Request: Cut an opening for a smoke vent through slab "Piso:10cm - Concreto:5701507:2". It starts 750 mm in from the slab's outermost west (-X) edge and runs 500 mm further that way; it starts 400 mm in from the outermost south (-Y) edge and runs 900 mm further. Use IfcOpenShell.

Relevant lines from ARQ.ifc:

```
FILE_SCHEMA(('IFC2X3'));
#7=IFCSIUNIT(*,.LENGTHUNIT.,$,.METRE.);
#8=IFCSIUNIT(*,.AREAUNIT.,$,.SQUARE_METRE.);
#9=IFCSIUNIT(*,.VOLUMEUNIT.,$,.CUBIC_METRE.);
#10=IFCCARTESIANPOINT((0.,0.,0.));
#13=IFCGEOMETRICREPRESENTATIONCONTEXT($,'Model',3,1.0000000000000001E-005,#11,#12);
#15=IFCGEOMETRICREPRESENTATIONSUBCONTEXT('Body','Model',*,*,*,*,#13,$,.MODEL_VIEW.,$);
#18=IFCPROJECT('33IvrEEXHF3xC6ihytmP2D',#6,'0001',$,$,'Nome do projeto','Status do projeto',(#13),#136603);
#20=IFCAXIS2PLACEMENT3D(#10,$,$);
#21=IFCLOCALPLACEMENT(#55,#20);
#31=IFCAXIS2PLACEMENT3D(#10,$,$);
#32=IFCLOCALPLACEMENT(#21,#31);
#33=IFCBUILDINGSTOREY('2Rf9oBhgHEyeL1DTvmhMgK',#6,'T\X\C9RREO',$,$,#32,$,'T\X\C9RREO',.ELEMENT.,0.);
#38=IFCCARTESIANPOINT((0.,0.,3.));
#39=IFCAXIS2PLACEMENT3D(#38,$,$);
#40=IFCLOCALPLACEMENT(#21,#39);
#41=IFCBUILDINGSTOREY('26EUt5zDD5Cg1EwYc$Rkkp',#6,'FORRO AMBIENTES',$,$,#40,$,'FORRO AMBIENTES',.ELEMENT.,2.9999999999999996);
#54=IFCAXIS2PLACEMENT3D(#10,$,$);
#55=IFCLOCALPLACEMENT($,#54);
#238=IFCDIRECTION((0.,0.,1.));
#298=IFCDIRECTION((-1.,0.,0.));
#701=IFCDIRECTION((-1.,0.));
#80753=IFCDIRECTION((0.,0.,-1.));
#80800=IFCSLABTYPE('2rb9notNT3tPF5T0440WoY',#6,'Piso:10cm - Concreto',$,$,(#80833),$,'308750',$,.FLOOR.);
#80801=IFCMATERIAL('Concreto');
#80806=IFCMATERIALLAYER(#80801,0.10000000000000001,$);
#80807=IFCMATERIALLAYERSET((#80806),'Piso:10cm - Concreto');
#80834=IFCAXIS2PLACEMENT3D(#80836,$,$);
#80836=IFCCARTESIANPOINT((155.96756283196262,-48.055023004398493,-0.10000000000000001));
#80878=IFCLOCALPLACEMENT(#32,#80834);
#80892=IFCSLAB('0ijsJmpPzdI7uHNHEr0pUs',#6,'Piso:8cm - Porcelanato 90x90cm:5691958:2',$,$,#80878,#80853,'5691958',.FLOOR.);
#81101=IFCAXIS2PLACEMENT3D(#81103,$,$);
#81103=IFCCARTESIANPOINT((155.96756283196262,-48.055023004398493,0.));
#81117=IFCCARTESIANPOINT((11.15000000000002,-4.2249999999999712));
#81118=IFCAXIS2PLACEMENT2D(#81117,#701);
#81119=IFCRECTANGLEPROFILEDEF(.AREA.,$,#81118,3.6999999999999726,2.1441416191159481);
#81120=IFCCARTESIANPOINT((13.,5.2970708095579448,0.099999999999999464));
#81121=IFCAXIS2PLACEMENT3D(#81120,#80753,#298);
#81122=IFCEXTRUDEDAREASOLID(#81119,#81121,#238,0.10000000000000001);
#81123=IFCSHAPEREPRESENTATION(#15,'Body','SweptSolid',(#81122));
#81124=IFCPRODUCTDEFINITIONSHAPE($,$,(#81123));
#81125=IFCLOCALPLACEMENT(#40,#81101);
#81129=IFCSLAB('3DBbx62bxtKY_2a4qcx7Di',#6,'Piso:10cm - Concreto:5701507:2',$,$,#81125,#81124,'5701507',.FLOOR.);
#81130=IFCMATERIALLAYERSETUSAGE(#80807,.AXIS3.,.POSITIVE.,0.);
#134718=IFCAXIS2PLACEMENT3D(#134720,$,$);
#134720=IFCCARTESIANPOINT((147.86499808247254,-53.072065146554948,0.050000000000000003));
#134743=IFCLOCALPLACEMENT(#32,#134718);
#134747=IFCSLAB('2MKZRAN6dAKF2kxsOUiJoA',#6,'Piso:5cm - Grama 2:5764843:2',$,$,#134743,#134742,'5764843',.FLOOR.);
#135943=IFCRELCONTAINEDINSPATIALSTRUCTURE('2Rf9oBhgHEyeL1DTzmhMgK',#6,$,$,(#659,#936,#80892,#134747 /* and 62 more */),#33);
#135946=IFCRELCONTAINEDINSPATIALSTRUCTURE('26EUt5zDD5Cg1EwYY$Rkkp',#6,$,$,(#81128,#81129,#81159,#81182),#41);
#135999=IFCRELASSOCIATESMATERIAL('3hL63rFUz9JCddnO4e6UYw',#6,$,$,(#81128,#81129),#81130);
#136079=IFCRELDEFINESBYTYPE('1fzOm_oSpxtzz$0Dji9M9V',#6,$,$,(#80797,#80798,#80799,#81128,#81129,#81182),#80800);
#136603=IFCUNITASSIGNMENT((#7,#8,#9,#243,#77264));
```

```python
import numpy as np
import ifcopenshell
import ifcopenshell.api.feature
import ifcopenshell.api.geometry
import ifcopenshell.api.root
import ifcopenshell.geom
import ifcopenshell.util.placement
import ifcopenshell.util.representation
import ifcopenshell.util.shape
import ifcopenshell.util.unit

model = ifcopenshell.open("ARQ.ifc")
unit_scale = ifcopenshell.util.unit.calculate_unit_scale(model)
settings = ifcopenshell.geom.settings()


def volume(element):
    """Net volume in cubic metres, openings subtracted."""
    shape = ifcopenshell.geom.create_shape(settings, element)
    return ifcopenshell.util.shape.get_volume(shape.geometry)


slab = model.by_id(81129)
before = volume(slab)

# Extent in the slab's own axes, in metres. The edges named are its -X and -Y sides.
slab_shape = ifcopenshell.geom.create_shape(settings, slab)
vertices = ifcopenshell.util.shape.get_vertices(slab_shape.geometry)
x_min, y_min, bottom = vertices.min(axis=0)
top = vertices[:, 2].max()

opening = ifcopenshell.api.root.create_entity(model, ifc_class="IfcOpeningElement", name="Smoke vent opening")
context = ifcopenshell.util.representation.get_context(model, "Model", "Body", "MODEL_VIEW")
width, depth = 0.5, 0.9
outline = [(0.0, 0.0), (width, 0.0), (width, depth), (0.0, depth), (0.0, 0.0)]
# Overshoot both faces by 50 mm so the cut is clean.
shape = ifcopenshell.api.geometry.add_slab_representation(
    model, context=context, depth=top - bottom + 0.1, polyline=outline
)
ifcopenshell.api.geometry.assign_representation(model, product=opening, representation=shape)

matrix = ifcopenshell.util.placement.get_local_placement(slab.ObjectPlacement)
matrix[:, 3] = matrix @ np.append(np.array([x_min + 0.75, y_min + 0.4, bottom - 0.05]) / unit_scale, 1.0)
ifcopenshell.api.geometry.edit_object_placement(model, product=opening, matrix=matrix, is_si=False)
ifcopenshell.api.feature.add_feature(model, feature=opening, element=slab)

after = volume(slab)

print(f"slab volume {before:.3f} -> {after:.3f} m3")

model.write("ARQ_updated.ifc")
```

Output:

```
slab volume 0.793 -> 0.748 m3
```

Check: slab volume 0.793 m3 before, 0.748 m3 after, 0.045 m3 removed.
